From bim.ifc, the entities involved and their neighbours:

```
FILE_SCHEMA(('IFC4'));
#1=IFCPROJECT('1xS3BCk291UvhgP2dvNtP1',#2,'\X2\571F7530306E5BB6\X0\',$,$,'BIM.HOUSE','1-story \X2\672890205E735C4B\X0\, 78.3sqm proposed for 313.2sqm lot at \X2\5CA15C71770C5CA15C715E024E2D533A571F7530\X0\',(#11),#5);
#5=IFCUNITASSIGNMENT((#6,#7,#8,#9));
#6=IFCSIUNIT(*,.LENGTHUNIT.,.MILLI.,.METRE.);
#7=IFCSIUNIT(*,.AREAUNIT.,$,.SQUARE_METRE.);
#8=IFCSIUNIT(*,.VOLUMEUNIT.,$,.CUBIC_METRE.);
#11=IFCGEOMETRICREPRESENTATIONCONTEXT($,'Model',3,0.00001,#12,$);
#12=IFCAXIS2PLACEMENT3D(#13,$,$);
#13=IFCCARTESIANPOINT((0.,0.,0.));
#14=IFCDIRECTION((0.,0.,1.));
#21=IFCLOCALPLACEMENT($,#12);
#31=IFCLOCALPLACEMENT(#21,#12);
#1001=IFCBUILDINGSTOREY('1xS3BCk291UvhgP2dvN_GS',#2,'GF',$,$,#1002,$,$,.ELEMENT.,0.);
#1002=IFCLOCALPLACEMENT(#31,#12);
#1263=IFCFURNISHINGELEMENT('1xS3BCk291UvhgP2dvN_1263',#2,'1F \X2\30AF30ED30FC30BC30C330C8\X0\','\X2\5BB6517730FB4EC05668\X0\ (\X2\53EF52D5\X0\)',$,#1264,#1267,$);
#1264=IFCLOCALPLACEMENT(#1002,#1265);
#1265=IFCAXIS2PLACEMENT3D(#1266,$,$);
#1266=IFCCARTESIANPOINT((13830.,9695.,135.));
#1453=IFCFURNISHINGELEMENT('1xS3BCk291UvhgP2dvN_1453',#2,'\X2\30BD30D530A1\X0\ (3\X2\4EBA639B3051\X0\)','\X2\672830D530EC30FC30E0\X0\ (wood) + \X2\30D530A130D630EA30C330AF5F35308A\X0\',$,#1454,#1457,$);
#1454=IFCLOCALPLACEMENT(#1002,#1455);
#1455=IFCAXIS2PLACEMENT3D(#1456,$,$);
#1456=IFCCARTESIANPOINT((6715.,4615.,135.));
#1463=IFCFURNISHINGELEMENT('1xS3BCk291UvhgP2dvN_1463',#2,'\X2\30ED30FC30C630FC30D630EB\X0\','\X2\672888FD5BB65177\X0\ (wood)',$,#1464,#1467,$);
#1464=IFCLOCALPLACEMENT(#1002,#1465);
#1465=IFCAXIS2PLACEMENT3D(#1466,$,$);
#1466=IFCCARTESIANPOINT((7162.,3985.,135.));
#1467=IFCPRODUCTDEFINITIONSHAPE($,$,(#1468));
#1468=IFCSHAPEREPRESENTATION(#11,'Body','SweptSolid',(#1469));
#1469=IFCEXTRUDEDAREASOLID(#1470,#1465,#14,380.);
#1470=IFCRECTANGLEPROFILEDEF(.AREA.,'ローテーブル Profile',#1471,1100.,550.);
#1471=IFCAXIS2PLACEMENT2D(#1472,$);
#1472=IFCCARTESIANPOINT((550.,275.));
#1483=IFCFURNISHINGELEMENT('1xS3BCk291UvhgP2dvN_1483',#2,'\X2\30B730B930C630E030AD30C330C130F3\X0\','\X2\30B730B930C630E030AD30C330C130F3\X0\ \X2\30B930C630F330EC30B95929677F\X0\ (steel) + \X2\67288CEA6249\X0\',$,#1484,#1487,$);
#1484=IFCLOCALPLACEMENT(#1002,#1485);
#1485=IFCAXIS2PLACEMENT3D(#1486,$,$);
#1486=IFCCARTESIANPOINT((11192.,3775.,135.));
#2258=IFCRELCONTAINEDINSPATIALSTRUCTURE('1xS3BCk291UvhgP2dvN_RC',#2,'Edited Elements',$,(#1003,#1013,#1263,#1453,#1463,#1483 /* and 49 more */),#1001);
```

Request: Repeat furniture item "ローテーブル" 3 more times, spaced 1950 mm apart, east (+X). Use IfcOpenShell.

```python
import numpy as np
import ifcopenshell
import ifcopenshell.api.geometry
import ifcopenshell.api.root
import ifcopenshell.util.element
import ifcopenshell.util.placement
import ifcopenshell.util.unit

model = ifcopenshell.open("bim.ifc")
unit_scale = ifcopenshell.util.unit.calculate_unit_scale(model)


def reuse_history(source, copy):
    """copy_class also copies each property set's owner history, people and application; keep the originals."""
    for rel in copy.IsDefinedBy:
        if rel.is_a("IfcRelDefinesByProperties") and (history := rel.RelatingPropertyDefinition.OwnerHistory):
            rel.RelatingPropertyDefinition.OwnerHistory = source.OwnerHistory
            ifcopenshell.util.element.remove_deep2(model, history)


source = model.by_guid("1xS3BCk291UvhgP2dvN_1463")
base = ifcopenshell.util.placement.get_local_placement(source.ObjectPlacement)
step = np.array([1.0, 0.0, 0.0]) * 1.95 / unit_scale

for i in range(1, 4):
    copy = ifcopenshell.api.root.copy_class(model, product=source)
    copy.Representation = ifcopenshell.util.element.copy_deep(
        model, source.Representation, exclude=["IfcGeometricRepresentationContext", "IfcRepresentationMap"]
    )
    reuse_history(source, copy)
    matrix = base.copy()
    matrix[:3, 3] += i * step
    print("added at", matrix[:3, 3].round(3) + 0.0)
    ifcopenshell.api.geometry.edit_object_placement(model, product=copy, matrix=matrix, is_si=False)

model.write("bim_rev.ifc")
```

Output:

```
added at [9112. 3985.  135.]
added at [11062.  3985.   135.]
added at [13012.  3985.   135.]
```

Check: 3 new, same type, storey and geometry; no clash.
